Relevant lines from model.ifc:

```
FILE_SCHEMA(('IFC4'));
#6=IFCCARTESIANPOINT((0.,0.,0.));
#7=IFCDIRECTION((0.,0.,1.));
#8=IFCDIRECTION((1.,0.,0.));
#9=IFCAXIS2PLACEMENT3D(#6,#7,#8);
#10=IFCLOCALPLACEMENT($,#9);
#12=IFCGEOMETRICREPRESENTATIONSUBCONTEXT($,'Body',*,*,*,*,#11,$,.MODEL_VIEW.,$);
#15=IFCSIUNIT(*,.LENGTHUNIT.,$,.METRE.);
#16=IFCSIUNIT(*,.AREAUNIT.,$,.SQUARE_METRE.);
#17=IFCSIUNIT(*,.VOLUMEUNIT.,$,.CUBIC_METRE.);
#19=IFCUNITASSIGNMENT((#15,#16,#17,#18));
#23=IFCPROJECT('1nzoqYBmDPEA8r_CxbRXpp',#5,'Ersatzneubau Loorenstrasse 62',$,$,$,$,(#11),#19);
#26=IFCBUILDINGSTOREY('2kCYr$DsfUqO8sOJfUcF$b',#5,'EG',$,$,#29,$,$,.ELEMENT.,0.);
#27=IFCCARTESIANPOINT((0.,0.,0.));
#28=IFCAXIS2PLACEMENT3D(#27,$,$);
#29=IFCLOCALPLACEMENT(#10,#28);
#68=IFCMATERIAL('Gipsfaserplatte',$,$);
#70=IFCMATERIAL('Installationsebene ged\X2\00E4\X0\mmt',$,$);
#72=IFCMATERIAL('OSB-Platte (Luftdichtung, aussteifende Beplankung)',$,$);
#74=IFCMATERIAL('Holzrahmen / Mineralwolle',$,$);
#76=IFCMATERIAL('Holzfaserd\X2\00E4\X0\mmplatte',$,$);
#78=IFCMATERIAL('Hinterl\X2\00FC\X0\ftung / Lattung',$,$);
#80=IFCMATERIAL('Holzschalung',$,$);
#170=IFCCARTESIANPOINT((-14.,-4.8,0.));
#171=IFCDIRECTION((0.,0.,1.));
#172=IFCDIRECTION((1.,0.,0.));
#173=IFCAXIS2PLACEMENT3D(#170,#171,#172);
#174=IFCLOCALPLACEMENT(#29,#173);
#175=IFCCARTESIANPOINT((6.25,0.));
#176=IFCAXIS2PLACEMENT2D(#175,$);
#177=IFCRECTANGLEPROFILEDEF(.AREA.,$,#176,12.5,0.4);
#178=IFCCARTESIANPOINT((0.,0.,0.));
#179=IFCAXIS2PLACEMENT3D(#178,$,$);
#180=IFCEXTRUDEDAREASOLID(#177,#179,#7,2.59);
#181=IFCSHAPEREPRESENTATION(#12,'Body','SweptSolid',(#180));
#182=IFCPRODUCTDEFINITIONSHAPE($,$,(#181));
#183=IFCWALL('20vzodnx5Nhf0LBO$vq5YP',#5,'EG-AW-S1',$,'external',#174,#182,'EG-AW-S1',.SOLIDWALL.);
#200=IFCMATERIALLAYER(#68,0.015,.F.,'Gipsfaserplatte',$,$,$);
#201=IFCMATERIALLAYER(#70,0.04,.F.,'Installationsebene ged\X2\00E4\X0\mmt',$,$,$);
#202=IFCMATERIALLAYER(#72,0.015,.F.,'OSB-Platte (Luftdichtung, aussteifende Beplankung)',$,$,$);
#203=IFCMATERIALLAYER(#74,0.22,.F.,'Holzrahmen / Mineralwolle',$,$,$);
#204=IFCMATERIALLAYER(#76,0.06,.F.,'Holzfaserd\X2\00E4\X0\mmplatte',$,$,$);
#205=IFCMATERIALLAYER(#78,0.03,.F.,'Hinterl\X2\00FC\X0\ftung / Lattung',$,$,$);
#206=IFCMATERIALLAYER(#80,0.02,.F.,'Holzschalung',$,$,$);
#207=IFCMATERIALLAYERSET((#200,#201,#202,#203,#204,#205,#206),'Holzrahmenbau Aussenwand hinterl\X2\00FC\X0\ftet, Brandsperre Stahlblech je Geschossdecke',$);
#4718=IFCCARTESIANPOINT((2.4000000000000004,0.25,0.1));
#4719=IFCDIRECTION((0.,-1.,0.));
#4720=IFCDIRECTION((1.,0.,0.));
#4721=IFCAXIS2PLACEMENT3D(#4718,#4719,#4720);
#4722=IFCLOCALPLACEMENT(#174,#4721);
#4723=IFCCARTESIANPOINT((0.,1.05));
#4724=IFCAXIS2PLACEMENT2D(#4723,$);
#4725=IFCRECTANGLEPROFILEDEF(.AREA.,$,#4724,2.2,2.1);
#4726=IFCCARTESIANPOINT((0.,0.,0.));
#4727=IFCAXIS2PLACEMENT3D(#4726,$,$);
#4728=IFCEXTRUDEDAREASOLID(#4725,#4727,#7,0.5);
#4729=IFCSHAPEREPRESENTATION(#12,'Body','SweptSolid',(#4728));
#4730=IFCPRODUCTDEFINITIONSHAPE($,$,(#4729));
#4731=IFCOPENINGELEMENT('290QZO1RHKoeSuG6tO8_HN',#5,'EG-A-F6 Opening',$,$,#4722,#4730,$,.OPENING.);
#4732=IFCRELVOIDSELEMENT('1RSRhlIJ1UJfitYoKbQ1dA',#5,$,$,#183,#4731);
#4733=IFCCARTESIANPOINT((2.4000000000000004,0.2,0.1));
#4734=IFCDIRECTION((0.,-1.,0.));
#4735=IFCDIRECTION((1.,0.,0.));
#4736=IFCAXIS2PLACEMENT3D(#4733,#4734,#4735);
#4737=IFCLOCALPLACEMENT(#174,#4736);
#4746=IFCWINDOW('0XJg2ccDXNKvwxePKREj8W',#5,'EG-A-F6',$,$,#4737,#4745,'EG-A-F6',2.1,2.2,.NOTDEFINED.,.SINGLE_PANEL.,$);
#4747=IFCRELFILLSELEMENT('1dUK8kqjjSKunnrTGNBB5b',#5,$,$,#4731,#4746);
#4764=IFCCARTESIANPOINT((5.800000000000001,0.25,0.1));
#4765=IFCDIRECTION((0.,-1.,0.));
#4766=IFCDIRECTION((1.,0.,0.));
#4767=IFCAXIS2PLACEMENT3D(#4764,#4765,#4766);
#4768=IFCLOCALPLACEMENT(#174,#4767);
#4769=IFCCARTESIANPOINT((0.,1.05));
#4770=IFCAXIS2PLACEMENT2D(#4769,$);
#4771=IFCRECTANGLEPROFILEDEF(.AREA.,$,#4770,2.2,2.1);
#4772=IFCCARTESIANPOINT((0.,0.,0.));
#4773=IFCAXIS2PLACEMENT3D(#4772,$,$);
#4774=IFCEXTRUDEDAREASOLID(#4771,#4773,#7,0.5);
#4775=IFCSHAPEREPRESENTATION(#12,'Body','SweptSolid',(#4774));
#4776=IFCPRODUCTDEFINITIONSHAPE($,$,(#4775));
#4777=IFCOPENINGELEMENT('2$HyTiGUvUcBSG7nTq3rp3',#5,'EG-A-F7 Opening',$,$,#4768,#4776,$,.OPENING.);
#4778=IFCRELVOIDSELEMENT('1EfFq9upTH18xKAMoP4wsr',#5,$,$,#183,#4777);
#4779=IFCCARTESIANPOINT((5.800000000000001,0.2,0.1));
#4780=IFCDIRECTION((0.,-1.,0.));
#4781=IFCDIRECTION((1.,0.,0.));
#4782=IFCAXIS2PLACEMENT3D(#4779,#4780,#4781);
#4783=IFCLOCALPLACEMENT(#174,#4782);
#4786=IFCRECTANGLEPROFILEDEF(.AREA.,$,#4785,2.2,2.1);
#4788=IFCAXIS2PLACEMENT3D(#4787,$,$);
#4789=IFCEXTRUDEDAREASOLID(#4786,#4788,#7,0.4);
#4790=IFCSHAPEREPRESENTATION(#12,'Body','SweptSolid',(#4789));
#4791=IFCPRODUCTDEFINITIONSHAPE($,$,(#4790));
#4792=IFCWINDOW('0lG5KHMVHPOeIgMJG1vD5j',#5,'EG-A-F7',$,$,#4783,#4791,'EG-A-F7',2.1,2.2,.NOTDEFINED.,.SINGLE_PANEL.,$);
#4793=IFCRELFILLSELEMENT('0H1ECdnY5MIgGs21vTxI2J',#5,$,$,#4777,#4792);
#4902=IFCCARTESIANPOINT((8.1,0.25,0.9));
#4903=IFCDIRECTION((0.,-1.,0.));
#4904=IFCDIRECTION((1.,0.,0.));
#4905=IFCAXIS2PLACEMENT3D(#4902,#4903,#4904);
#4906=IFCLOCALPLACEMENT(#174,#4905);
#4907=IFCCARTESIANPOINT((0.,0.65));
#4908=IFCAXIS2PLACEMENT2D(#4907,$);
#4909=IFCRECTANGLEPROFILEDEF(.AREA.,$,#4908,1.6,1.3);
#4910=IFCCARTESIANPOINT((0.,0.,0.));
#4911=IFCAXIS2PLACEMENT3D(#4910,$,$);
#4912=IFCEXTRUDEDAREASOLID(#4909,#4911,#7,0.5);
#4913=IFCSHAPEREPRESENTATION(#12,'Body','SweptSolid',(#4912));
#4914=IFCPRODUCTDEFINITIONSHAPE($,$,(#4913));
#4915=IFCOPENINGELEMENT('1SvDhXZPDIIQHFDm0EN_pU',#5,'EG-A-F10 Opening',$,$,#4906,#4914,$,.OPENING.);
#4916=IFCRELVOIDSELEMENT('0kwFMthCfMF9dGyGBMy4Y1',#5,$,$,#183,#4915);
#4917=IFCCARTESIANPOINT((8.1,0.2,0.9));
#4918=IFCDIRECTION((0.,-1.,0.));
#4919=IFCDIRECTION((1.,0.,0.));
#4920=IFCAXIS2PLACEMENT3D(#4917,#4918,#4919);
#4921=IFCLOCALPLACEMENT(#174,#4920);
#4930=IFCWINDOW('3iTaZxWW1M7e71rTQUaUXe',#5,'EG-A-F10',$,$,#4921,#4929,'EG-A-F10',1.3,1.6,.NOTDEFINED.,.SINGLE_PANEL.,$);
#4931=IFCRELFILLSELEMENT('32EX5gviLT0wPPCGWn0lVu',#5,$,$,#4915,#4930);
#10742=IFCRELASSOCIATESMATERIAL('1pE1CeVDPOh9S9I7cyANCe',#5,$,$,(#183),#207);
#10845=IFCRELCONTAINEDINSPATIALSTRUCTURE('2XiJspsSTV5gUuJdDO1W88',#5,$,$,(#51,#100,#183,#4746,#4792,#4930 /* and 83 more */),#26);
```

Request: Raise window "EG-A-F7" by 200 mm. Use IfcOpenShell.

```python
import numpy as np
import ifcopenshell
import ifcopenshell.api.geometry
import ifcopenshell.util.placement
import ifcopenshell.util.unit

model = ifcopenshell.open("model.ifc")
unit_scale = ifcopenshell.util.unit.calculate_unit_scale(model)

window = model.by_guid("0lG5KHMVHPOeIgMJG1vD5j")
opening = window.FillsVoids[0].RelatingOpeningElement
dz = 0.2 / unit_scale

shift = np.array([0.0, 0.0, dz])
# The window is not placed relative to its opening, so move both.
for product in (opening, window):
    matrix = ifcopenshell.util.placement.get_local_placement(product.ObjectPlacement)
    matrix[:3, 3] += shift
    ifcopenshell.api.geometry.edit_object_placement(model, product=product, matrix=matrix, is_si=False)

print(f"moved by {dz * unit_scale:+.3f} m")

model.write("model_updated.ifc")
```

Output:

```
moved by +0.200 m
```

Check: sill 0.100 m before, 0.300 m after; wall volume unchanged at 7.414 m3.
